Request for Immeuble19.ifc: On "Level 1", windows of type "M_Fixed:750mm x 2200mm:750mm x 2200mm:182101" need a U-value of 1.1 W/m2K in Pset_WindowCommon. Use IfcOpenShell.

First a look at what the model holds.

```python
import ifcopenshell
import ifcopenshell.util.element

model = ifcopenshell.open("Immeuble19.ifc")
print(model.schema)
storey = next(s for s in model.by_type("IfcBuildingStorey") if s.Name == "Level 1")
windows = [e for e in ifcopenshell.util.element.get_decomposition(storey) if e.is_a("IfcWindow")]
seen = {}
for e in windows:
    element_type = ifcopenshell.util.element.get_type(e)
    key = (element_type.Name if element_type != e and element_type else None, ifcopenshell.util.element.get_pset(e, "Pset_WindowCommon", "ThermalTransmittance"))
    seen[key] = seen.get(key, 0) + 1
for (name, value), count in sorted(seen.items(), key=str):
    print(count, "x", name, "|", value)
```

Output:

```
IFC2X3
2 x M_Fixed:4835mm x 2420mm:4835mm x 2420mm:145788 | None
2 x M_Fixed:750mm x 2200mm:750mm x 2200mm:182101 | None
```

```python
import ifcopenshell
import ifcopenshell.api.pset
import ifcopenshell.util.element

model = ifcopenshell.open("Immeuble19.ifc")

storey = next(s for s in model.by_type("IfcBuildingStorey") if s.Name == "Level 1")
windows = [e for e in ifcopenshell.util.element.get_decomposition(storey) if e.is_a("IfcWindow")]

count = 0
for e in windows:
    element_type = ifcopenshell.util.element.get_type(e)
    if element_type in (None, e) or element_type.Name != "M_Fixed:750mm x 2200mm:750mm x 2200mm:182101":
        continue
    # add_pset returns the element's existing set when there is one.
    pset = ifcopenshell.api.pset.add_pset(model, product=e, name="Pset_WindowCommon")
    ifcopenshell.api.pset.edit_pset(model, pset=pset, properties={"ThermalTransmittance": 1.1})
    count += 1

print(count, "windows updated")

model.write("Immeuble19-out.ifc")
```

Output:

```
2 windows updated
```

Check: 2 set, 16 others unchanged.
